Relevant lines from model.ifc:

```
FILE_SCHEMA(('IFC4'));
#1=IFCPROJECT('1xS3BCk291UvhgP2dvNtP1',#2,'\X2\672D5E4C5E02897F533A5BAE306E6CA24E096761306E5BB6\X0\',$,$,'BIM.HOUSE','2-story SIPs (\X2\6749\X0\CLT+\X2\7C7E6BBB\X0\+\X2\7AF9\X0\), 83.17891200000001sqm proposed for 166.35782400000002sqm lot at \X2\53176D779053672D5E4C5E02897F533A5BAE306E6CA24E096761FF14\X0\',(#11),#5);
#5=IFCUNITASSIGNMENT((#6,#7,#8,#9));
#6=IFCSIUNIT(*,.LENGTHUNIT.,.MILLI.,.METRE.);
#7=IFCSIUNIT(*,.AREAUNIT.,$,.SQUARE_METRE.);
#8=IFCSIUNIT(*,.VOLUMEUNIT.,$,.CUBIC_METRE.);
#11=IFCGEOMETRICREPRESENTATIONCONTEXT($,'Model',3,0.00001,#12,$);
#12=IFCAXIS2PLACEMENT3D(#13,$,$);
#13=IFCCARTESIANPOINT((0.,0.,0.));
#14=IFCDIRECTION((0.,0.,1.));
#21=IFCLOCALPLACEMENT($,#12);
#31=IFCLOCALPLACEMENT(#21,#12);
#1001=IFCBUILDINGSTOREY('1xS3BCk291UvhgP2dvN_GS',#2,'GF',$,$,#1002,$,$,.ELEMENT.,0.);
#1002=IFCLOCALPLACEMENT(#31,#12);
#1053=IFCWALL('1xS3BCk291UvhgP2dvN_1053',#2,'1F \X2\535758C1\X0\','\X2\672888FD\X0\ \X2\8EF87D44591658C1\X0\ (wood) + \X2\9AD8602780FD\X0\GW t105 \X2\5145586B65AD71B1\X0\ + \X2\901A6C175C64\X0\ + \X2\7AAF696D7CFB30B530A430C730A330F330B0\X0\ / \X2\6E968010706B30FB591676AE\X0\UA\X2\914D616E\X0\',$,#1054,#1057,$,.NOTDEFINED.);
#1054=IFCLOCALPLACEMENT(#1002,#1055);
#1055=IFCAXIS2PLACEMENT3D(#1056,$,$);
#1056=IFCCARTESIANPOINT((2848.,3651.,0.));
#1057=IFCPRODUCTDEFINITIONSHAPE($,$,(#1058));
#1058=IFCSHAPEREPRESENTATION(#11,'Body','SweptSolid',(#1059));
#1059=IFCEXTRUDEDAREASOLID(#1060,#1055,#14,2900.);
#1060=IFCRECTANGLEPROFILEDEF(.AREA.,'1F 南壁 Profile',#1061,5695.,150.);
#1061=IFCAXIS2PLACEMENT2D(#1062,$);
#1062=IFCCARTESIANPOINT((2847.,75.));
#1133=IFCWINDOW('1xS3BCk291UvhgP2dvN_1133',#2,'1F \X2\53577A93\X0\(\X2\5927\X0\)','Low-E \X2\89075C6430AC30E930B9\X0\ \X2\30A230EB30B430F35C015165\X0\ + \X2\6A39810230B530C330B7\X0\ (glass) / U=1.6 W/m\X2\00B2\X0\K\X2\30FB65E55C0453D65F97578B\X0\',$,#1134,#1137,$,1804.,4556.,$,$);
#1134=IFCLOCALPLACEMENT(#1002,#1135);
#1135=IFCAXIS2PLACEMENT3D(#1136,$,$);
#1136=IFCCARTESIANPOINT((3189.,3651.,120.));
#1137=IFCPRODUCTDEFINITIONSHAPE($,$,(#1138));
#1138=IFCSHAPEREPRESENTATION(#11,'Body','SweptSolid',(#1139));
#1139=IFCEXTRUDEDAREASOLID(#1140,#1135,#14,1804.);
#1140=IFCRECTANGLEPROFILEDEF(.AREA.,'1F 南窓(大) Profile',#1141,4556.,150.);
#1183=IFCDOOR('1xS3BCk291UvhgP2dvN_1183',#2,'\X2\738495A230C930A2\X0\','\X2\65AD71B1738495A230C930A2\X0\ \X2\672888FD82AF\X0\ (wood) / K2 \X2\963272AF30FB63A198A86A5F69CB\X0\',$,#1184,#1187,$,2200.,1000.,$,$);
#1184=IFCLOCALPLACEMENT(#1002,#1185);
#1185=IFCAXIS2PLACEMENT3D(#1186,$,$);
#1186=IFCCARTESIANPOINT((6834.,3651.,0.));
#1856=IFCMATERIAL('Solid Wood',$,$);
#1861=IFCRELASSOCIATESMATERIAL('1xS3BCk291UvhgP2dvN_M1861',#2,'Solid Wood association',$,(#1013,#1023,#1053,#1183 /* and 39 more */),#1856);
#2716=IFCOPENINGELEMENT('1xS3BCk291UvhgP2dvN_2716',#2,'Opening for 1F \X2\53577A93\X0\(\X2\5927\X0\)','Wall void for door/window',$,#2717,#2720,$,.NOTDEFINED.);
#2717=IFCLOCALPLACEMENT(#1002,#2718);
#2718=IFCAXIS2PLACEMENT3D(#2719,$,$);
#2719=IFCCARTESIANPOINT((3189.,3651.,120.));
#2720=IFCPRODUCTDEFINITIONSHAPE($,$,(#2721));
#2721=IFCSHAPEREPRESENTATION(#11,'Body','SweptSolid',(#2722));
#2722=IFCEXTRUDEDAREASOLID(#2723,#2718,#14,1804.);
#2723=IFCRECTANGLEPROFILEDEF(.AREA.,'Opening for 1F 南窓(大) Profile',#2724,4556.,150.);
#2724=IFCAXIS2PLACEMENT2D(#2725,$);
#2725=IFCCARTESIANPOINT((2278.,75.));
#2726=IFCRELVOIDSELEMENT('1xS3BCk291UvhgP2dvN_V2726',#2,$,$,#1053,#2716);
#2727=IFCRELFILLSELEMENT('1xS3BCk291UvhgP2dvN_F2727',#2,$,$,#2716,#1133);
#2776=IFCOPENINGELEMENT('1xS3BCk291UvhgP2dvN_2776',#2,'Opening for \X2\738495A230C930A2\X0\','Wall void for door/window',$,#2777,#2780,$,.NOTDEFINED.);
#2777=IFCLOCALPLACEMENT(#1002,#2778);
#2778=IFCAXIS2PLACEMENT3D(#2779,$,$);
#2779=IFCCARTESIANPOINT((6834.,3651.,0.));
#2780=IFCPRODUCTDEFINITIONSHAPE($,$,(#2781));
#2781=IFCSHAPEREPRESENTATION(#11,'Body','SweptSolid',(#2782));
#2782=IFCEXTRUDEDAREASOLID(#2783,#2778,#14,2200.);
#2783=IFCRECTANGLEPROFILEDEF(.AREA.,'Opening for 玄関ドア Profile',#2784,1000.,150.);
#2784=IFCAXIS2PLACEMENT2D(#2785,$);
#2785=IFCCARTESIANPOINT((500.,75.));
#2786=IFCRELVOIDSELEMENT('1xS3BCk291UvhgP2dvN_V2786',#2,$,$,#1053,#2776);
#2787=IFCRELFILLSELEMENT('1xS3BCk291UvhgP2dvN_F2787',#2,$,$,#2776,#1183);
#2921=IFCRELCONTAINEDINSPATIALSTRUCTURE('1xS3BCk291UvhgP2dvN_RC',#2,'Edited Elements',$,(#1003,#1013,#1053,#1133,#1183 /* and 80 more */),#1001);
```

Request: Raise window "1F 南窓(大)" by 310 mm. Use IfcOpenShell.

```python
import numpy as np
import ifcopenshell
import ifcopenshell.api.geometry
import ifcopenshell.util.placement
import ifcopenshell.util.unit

model = ifcopenshell.open("model.ifc")
unit_scale = ifcopenshell.util.unit.calculate_unit_scale(model)

window = model.by_id(1133)
opening = window.FillsVoids[0].RelatingOpeningElement
dz = 0.31 / unit_scale

shift = np.array([0.0, 0.0, dz])
# The window is not placed relative to its opening, so move both.
for product in (opening, window):
    matrix = ifcopenshell.util.placement.get_local_placement(product.ObjectPlacement)
    matrix[:3, 3] += shift
    ifcopenshell.api.geometry.edit_object_placement(model, product=product, matrix=matrix, is_si=False)

print(f"moved by {dz * unit_scale:+.3f} m")

model.write("model-out.ifc")
```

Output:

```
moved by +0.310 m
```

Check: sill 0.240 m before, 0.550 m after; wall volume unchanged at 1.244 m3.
